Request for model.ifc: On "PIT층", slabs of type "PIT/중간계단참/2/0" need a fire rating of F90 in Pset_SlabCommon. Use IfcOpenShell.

First a look at what the model holds.

```python
import ifcopenshell
import ifcopenshell.util.element

model = ifcopenshell.open("model.ifc")
print(model.schema)
storey = next(s for s in model.by_type("IfcBuildingStorey") if s.Name == "PIT층")
slabs = [e for e in ifcopenshell.util.element.get_decomposition(storey) if e.is_a("IfcSlab")]
seen = {}
for e in slabs:
    element_type = ifcopenshell.util.element.get_type(e)
    key = (element_type.Name if element_type != e and element_type else None, ifcopenshell.util.element.get_pset(e, "Pset_SlabCommon", "FireRating"))
    seen[key] = seen.get(key, 0) + 1
for (name, value), count in sorted(seen.items(), key=str):
    print(count, "x", name, "|", value)
```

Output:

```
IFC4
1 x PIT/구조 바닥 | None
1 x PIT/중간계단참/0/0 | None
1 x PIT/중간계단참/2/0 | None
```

```python
import ifcopenshell
import ifcopenshell.api.pset
import ifcopenshell.util.element

model = ifcopenshell.open("model.ifc")

storey = next(s for s in model.by_type("IfcBuildingStorey") if s.Name == "PIT층")
slabs = [e for e in ifcopenshell.util.element.get_decomposition(storey) if e.is_a("IfcSlab")]

count = 0
for e in slabs:
    element_type = ifcopenshell.util.element.get_type(e)
    if element_type in (None, e) or element_type.Name != "PIT/중간계단참/2/0":
        continue
    # add_pset returns the element's existing set when there is one.
    pset = ifcopenshell.api.pset.add_pset(model, product=e, name="Pset_SlabCommon")
    ifcopenshell.api.pset.edit_pset(model, pset=pset, properties={"FireRating": "F90"})
    count += 1

print(count, "slabs updated")

model.write("model_updated.ifc")
```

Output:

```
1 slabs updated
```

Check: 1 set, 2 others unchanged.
